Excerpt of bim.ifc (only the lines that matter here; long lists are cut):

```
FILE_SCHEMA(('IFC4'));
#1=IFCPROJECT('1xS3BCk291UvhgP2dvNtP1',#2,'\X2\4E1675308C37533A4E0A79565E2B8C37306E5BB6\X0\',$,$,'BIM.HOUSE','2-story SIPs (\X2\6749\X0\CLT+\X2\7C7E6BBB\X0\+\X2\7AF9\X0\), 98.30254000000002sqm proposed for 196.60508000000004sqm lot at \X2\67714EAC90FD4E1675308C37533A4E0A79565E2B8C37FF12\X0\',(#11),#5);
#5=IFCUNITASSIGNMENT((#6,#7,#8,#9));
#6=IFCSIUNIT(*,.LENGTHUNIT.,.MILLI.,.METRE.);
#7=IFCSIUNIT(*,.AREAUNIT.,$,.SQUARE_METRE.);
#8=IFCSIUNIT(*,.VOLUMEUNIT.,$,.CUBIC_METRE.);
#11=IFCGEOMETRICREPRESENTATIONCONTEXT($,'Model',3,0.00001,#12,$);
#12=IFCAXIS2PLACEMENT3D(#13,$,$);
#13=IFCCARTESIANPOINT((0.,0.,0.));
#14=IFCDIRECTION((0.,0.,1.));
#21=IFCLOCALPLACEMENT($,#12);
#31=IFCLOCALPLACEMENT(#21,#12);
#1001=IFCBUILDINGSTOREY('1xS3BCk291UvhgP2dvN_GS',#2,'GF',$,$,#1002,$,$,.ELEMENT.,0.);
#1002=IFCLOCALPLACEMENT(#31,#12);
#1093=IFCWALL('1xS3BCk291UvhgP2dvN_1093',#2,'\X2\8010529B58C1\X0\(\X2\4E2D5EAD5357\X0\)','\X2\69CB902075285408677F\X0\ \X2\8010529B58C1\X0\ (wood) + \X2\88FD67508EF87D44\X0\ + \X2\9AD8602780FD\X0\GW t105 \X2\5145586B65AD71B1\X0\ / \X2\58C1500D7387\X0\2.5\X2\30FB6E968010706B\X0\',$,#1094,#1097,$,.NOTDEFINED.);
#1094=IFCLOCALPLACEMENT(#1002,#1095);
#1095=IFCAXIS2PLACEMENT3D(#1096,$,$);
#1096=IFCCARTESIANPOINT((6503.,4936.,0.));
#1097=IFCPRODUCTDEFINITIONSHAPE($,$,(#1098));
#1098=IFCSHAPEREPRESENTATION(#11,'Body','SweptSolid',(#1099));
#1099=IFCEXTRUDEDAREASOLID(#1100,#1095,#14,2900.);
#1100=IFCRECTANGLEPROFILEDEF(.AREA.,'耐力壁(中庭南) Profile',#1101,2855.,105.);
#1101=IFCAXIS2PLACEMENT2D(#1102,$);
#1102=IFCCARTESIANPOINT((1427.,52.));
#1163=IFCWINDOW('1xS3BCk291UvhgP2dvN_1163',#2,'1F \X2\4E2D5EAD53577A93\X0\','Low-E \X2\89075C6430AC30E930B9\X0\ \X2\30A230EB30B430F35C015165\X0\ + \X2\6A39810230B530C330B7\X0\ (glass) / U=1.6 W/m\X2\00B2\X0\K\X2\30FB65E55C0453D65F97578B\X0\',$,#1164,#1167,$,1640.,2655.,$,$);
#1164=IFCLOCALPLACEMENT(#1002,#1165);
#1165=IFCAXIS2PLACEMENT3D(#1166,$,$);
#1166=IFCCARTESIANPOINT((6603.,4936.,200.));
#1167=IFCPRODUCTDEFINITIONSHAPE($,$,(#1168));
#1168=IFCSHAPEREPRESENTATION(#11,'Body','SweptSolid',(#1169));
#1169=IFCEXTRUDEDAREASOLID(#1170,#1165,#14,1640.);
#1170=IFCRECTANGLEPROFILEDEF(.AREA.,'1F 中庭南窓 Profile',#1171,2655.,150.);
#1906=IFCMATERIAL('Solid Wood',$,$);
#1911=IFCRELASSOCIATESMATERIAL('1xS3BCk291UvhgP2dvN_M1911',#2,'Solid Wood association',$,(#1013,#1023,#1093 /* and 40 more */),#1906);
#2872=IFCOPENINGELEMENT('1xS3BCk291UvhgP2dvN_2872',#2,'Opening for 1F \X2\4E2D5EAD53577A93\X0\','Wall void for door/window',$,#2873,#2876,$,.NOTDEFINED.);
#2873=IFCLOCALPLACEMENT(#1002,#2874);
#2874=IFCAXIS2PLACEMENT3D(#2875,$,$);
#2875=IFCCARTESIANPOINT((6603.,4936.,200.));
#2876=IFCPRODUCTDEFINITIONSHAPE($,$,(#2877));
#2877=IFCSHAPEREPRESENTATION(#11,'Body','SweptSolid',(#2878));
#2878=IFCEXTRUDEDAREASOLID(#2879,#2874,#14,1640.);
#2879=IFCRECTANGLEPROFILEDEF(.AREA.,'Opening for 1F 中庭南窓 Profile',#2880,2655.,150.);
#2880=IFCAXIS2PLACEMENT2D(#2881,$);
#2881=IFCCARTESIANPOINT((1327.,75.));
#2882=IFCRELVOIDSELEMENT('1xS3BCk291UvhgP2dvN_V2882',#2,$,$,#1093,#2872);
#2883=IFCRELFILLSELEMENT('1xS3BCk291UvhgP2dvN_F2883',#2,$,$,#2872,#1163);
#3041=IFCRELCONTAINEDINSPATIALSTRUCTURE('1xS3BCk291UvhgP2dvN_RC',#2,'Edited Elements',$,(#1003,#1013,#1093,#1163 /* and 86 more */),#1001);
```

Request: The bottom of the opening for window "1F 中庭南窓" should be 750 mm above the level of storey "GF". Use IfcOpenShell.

```python
import numpy as np
import ifcopenshell
import ifcopenshell.api.geometry
import ifcopenshell.geom
import ifcopenshell.util.element
import ifcopenshell.util.placement
import ifcopenshell.util.shape
import ifcopenshell.util.unit

model = ifcopenshell.open("bim.ifc")
unit_scale = ifcopenshell.util.unit.calculate_unit_scale(model)

window = model.by_guid("1xS3BCk291UvhgP2dvN_1163")
opening = window.FillsVoids[0].RelatingOpeningElement
storey = ifcopenshell.util.element.get_container(window, ifc_class="IfcBuildingStorey")
level = ifcopenshell.util.placement.get_local_placement(storey.ObjectPlacement)[2, 3]

# The opening's origin need not be at the sill, so measure its lowest point.
shape = ifcopenshell.geom.create_shape(ifcopenshell.geom.settings(), opening)
bottom = ifcopenshell.util.shape.get_shape_bottom_elevation(shape, shape.geometry) / unit_scale
dz = level + 0.75 / unit_scale - bottom

shift = np.array([0.0, 0.0, dz])
# The window is not placed relative to its opening, so move both.
for product in (opening, window):
    matrix = ifcopenshell.util.placement.get_local_placement(product.ObjectPlacement)
    matrix[:3, 3] += shift
    ifcopenshell.api.geometry.edit_object_placement(model, product=product, matrix=matrix, is_si=False)

print(f"moved by {dz * unit_scale:+.3f} m")

model.write("bim_rev.ifc")
```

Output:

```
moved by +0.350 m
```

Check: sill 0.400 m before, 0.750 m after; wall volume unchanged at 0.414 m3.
